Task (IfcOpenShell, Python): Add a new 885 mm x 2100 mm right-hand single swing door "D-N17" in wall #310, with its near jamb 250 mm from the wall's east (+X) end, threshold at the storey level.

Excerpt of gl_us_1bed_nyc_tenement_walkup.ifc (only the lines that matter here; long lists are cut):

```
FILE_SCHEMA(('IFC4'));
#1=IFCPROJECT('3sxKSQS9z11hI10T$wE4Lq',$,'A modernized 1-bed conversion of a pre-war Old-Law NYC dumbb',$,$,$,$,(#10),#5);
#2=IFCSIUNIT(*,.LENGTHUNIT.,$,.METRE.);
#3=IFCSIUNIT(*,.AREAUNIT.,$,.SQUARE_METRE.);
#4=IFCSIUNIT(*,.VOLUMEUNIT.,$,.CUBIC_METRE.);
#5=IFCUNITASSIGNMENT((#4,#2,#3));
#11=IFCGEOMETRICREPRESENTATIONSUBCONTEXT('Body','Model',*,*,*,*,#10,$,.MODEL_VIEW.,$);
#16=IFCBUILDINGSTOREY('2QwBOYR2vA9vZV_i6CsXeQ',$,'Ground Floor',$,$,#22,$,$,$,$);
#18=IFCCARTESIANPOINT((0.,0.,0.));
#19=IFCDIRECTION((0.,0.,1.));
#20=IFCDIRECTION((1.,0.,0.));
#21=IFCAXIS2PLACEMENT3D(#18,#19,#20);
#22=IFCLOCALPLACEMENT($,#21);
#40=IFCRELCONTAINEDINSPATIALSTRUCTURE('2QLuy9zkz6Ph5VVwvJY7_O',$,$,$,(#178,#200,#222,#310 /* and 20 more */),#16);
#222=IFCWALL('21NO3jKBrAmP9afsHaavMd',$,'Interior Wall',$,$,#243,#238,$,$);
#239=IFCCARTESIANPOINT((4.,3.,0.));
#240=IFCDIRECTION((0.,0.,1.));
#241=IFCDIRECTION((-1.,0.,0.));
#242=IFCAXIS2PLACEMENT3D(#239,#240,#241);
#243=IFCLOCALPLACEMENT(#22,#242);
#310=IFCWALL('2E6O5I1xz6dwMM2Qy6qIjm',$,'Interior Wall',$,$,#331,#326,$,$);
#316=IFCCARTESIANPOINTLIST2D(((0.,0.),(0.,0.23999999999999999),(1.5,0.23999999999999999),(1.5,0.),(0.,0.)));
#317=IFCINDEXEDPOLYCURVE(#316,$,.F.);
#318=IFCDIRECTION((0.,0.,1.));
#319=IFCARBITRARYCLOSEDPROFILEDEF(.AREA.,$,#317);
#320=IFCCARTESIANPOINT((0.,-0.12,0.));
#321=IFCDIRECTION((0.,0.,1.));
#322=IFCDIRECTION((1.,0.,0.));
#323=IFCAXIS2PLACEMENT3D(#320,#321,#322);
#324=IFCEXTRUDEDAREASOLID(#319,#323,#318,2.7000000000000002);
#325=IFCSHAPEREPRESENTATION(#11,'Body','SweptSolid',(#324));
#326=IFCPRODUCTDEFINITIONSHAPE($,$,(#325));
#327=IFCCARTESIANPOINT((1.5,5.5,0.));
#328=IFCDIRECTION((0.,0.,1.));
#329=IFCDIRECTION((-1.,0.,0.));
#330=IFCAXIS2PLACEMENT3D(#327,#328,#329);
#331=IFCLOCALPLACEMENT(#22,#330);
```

```python
import numpy as np
import ifcopenshell
import ifcopenshell.api.feature
import ifcopenshell.api.geometry
import ifcopenshell.api.root
import ifcopenshell.api.spatial
import ifcopenshell.geom
import ifcopenshell.util.element
import ifcopenshell.util.placement
import ifcopenshell.util.representation
import ifcopenshell.util.shape
import ifcopenshell.util.unit

model = ifcopenshell.open("gl_us_1bed_nyc_tenement_walkup.ifc")
unit_scale = ifcopenshell.util.unit.calculate_unit_scale(model)
settings = ifcopenshell.geom.settings()


def volume(element):
    """Net volume in cubic metres, openings subtracted."""
    shape = ifcopenshell.geom.create_shape(settings, element)
    return ifcopenshell.util.shape.get_volume(shape.geometry)


wall = model.by_id(310)
storey = ifcopenshell.util.element.get_container(wall, ifc_class="IfcBuildingStorey")
context = ifcopenshell.util.representation.get_context(model, "Model", "Body", "MODEL_VIEW")
before = volume(wall)

width, height, from_end, sill = 0.885, 2.1, 0.25, 0.0  # metres

# The wall runs along its own X axis, and the end named is its -X end.
wall_shape = ifcopenshell.geom.create_shape(settings, wall)
x, y, z = ifcopenshell.util.shape.get_vertices(wall_shape.geometry).T
start = x.min() + from_end
face, thickness = float(y.min()), float(y.max() - y.min())
wall_matrix = ifcopenshell.util.placement.get_local_placement(wall.ObjectPlacement)
level = ifcopenshell.util.placement.get_local_placement(storey.ObjectPlacement)[2, 3]


def in_wall(x, y):
    """Placement at x, y metres in the wall's axes, at sill height."""
    matrix = wall_matrix.copy()
    matrix[:, 3] = wall_matrix @ np.array([x / unit_scale, y / unit_scale, 0.0, 1.0])
    matrix[2, 3] = level + sill / unit_scale
    return matrix


# Opening: a box that overshoots both wall faces by 50 mm.
opening = ifcopenshell.api.root.create_entity(model, ifc_class="IfcOpeningElement", predefined_type="OPENING")
box = ifcopenshell.api.geometry.add_wall_representation(
    model, context=context, length=width, height=height, thickness=thickness + 0.1
)
ifcopenshell.api.geometry.assign_representation(model, product=opening, representation=box)
ifcopenshell.api.geometry.edit_object_placement(model, product=opening, matrix=in_wall(start, face - 0.05), is_si=False)
ifcopenshell.api.feature.add_feature(model, feature=opening, element=wall)

door = ifcopenshell.api.root.create_entity(model, ifc_class="IfcDoor", name="D-N17", predefined_type="DOOR")
door.OverallWidth, door.OverallHeight = width / unit_scale, height / unit_scale
door.OperationType = "SINGLE_SWING_RIGHT"
body = ifcopenshell.api.geometry.add_door_representation(
    model,
    context=context,
    overall_width=door.OverallWidth,
    overall_height=door.OverallHeight,
    operation_type="SINGLE_SWING_RIGHT",
    lining_properties={"LiningDepth": thickness / unit_scale, "ThresholdDepth": thickness / unit_scale},
)
ifcopenshell.api.geometry.assign_representation(model, product=door, representation=body)
ifcopenshell.api.spatial.assign_container(model, products=[door], relating_structure=storey)
ifcopenshell.api.feature.add_filling(model, opening=opening, element=door)

# The lining spans the wall, so the door starts at the wall face.
ifcopenshell.api.geometry.edit_object_placement(model, product=door, matrix=in_wall(start, face), is_si=False)

after = volume(wall)

print(f"wall volume {before:.3f} -> {after:.3f} m3")

model.write("gl_us_1bed_nyc_tenement_walkup_edited.ifc")
```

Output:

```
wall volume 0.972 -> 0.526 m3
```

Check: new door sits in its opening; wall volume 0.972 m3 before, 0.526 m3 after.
